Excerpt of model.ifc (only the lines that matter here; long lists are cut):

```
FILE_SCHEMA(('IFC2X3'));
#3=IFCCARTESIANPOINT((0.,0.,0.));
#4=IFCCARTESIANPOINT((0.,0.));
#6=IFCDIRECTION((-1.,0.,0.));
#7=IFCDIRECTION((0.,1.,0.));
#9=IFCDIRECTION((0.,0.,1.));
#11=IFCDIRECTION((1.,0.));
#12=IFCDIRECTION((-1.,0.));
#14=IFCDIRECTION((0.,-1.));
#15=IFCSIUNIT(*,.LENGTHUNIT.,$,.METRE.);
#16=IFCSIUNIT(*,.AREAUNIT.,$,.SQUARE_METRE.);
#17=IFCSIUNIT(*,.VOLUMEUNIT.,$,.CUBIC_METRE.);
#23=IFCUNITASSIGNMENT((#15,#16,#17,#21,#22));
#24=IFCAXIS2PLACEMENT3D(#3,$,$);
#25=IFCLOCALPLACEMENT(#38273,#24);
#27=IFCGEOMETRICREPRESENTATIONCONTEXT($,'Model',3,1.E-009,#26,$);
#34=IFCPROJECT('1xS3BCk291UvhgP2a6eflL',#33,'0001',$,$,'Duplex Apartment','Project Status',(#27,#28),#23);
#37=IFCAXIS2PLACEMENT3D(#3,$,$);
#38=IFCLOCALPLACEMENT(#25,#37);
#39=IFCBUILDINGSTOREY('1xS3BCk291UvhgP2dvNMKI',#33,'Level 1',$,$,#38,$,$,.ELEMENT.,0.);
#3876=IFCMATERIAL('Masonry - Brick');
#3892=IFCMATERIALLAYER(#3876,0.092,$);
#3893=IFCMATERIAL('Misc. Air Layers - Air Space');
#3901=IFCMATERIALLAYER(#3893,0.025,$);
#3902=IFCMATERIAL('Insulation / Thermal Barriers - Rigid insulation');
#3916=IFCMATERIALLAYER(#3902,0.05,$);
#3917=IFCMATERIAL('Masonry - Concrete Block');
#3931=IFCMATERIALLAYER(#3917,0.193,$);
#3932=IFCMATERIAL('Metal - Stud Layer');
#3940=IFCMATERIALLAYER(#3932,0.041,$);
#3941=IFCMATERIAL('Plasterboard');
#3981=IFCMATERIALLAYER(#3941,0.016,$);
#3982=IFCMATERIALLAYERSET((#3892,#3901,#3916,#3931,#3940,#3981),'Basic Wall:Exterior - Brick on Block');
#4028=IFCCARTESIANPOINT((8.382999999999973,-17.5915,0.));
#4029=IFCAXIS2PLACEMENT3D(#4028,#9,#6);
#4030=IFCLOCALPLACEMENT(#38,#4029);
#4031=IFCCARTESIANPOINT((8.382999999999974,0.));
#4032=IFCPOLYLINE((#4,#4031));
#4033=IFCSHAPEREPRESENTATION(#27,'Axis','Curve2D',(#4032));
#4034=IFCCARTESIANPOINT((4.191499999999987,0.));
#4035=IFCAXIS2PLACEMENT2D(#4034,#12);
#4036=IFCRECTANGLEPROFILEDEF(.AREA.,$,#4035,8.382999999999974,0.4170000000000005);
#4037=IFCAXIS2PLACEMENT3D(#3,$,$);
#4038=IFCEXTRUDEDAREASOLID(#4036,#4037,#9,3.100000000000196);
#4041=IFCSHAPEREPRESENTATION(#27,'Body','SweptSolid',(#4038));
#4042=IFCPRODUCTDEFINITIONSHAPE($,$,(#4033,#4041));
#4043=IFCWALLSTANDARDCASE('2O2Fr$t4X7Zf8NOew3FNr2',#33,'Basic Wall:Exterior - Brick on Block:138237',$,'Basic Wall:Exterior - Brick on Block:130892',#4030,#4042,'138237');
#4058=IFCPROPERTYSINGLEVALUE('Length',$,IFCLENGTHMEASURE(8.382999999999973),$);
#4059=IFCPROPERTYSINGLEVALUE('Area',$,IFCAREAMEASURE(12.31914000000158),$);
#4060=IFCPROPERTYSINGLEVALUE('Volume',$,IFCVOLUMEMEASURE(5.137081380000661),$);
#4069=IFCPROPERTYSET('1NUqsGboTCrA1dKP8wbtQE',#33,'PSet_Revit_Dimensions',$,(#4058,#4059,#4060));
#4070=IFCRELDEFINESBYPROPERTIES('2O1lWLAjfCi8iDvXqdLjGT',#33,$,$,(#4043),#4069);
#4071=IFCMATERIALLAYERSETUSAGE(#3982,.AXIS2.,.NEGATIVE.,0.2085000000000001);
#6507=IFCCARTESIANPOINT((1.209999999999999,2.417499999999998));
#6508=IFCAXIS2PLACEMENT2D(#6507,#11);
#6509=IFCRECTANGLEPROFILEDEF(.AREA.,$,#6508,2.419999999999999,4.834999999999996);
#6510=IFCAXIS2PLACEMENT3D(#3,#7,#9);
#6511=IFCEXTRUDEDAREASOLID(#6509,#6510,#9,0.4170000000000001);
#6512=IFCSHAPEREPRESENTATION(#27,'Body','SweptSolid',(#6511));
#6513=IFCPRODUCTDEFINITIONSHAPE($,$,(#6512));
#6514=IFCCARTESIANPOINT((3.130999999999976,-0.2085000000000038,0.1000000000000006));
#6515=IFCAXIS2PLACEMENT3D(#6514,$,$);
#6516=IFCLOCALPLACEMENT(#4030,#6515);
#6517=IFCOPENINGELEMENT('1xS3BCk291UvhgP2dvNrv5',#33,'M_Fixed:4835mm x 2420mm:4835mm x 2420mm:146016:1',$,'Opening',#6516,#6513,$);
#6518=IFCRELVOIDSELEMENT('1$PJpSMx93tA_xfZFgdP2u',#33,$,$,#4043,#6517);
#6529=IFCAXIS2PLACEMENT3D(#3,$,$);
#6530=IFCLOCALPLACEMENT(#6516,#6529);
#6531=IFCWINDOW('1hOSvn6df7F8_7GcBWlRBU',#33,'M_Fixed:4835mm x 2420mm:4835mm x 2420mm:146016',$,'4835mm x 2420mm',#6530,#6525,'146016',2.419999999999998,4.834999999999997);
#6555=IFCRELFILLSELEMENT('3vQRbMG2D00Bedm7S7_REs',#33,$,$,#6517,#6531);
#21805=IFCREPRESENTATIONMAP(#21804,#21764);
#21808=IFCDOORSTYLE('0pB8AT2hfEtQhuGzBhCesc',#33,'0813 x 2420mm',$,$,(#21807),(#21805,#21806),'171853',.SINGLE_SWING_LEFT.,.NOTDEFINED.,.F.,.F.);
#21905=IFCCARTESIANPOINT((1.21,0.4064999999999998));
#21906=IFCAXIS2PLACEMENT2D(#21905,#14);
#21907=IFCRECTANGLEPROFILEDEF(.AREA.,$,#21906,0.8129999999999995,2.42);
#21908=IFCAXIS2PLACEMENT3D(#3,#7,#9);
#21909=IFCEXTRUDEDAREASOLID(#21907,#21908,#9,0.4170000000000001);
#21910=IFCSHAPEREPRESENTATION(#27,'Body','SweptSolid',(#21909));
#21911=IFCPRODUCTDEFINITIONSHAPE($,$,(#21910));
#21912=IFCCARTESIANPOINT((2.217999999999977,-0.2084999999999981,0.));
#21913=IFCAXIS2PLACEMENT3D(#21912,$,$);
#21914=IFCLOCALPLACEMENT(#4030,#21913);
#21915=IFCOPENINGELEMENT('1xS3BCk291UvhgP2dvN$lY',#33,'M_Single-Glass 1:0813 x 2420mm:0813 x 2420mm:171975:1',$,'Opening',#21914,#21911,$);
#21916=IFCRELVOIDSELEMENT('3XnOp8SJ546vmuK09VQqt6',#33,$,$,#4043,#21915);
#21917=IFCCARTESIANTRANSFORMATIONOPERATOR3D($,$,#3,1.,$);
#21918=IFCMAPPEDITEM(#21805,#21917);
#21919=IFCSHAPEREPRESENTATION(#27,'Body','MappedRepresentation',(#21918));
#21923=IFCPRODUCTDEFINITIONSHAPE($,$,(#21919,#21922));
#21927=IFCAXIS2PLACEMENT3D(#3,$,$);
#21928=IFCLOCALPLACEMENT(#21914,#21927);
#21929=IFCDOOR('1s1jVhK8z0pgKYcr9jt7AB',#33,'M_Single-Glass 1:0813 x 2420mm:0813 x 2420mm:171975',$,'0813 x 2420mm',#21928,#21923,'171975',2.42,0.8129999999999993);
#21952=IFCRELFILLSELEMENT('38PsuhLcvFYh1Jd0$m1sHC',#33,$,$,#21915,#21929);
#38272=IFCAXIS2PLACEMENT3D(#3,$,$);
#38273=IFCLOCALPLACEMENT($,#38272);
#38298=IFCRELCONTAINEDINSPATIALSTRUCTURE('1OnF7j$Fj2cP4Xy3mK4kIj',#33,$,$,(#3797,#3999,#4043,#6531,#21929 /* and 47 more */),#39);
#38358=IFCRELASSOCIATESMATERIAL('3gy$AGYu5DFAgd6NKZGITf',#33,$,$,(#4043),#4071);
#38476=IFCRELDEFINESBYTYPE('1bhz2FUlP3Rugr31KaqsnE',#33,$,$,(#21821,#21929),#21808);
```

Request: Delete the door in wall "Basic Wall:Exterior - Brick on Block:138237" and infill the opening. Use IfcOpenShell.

```python
import ifcopenshell
import ifcopenshell.api.feature
import ifcopenshell.api.pset
import ifcopenshell.api.root
import ifcopenshell.geom
import ifcopenshell.util.element
import ifcopenshell.util.shape
import ifcopenshell.util.unit

model = ifcopenshell.open("model.ifc")
area_scale = ifcopenshell.util.unit.calculate_unit_scale(model, "AREAUNIT")
volume_scale = ifcopenshell.util.unit.calculate_unit_scale(model, "VOLUMEUNIT")
settings = ifcopenshell.geom.settings()


def volume(element):
    """Net volume in cubic metres, openings subtracted."""
    shape = ifcopenshell.geom.create_shape(settings, element)
    return ifcopenshell.util.shape.get_volume(shape.geometry)


door = model.by_guid("1s1jVhK8z0pgKYcr9jt7AB")
opening = door.FillsVoids[0].RelatingOpeningElement
wall = opening.VoidsElements[0].RelatingBuildingElement
before = volume(wall)

ifcopenshell.api.root.remove_product(model, product=door)
ifcopenshell.api.feature.remove_feature(model, feature=opening)

after = volume(wall)
thickness = 0.417  # wall thickness in metres

# Update the wall's stored quantities.
pset = model.by_id(ifcopenshell.util.element.get_pset(wall, "PSet_Revit_Dimensions", should_inherit=False)["id"])
ifcopenshell.api.pset.edit_pset(model, pset=pset, properties={
    "Area": model.create_entity("IfcAreaMeasure", after / thickness / area_scale),
    "Volume": model.create_entity("IfcVolumeMeasure", after / volume_scale),
})

print(f"wall volume {before:.3f} -> {after:.3f} m3")

model.write("model_rev.ifc")
```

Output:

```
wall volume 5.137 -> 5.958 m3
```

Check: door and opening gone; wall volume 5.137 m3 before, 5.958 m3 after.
